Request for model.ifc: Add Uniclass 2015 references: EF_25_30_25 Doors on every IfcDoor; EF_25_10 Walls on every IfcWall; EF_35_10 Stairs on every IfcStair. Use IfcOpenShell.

First a look at what the model holds.

```python
import ifcopenshell

model = ifcopenshell.open("model.ifc")
print(model.schema)
print("classifications:", [c.Name for c in model.by_type("IfcClassification")])
for ifc_class in ("IfcDoor", "IfcRoof", "IfcStair", "IfcWall", "IfcWindow"):
    print(ifc_class, len(model.by_type(ifc_class)))
```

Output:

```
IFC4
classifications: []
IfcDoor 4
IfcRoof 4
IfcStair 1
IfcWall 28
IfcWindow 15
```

```python
import ifcopenshell
import ifcopenshell.api.classification

model = ifcopenshell.open("model.ifc")

system = ifcopenshell.api.classification.add_classification(model, classification="Uniclass 2015")

codes = {
    "IfcDoor": ("EF_25_30_25", "Doors"),
    "IfcWall": ("EF_25_10", "Walls"),
    "IfcStair": ("EF_35_10", "Stairs"),
}
for ifc_class, (code, name) in codes.items():
    products = model.by_type(ifc_class)
    ifcopenshell.api.classification.add_reference(
        model, products=products, classification=system, identification=code, name=name
    )
    print(code, len(products))

model.write("model_updated.ifc")
```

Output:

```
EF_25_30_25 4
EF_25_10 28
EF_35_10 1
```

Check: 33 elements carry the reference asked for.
